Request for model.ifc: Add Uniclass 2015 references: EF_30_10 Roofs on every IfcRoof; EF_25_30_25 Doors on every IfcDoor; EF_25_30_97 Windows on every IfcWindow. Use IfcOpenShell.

First a look at what the model holds.

```python
import ifcopenshell

model = ifcopenshell.open("model.ifc")
print(model.schema)
print("classifications:", [c.Name for c in model.by_type("IfcClassification")])
for ifc_class in ("IfcDoor", "IfcRoof", "IfcStair", "IfcWall", "IfcWindow"):
    print(ifc_class, len(model.by_type(ifc_class)))
```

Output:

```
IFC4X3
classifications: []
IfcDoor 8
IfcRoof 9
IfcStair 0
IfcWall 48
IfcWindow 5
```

```python
import ifcopenshell
import ifcopenshell.api.classification

model = ifcopenshell.open("model.ifc")

system = ifcopenshell.api.classification.add_classification(model, classification="Uniclass 2015")

codes = {
    "IfcRoof": ("EF_30_10", "Roofs"),
    "IfcDoor": ("EF_25_30_25", "Doors"),
    "IfcWindow": ("EF_25_30_97", "Windows"),
}
for ifc_class, (code, name) in codes.items():
    products = model.by_type(ifc_class)
    ifcopenshell.api.classification.add_reference(
        model, products=products, classification=system, identification=code, name=name
    )
    print(code, len(products))

model.write("model_edited.ifc")
```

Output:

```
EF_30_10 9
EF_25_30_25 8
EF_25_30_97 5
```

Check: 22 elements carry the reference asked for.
